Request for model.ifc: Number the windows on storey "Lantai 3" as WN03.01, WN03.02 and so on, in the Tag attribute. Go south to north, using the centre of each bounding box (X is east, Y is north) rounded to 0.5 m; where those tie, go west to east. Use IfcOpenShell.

First a look at what the model holds.

```python
import ifcopenshell
import ifcopenshell.util.element
import ifcopenshell.util.placement

model = ifcopenshell.open("model.ifc")
print(model.schema)
storey = next(s for s in model.by_type("IfcBuildingStorey") if s.Name == "Lantai 3")
windows = [e for e in ifcopenshell.util.element.get_decomposition(storey) if e.is_a("IfcWindow")]
for e in sorted(windows, key=lambda e: e.id()):
    origin = ifcopenshell.util.placement.get_local_placement(e.ObjectPlacement)[:3, 3]
    print(e.id(), e.Tag, e.Name, origin.round(2) + 0.0, sep=" | ")
```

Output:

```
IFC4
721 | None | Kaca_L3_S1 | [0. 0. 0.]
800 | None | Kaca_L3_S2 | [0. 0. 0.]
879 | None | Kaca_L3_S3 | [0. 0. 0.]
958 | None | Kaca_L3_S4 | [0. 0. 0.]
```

```python
import ifcopenshell
import ifcopenshell.geom
import ifcopenshell.util.element
import ifcopenshell.util.shape

model = ifcopenshell.open("model.ifc")
settings = ifcopenshell.geom.settings()
settings.set("use-world-coords", True)


def centre(element):
    shape = ifcopenshell.geom.create_shape(settings, element)
    return ifcopenshell.util.shape.get_bbox_centroid(shape.geometry)


storey = next(s for s in model.by_type("IfcBuildingStorey") if s.Name == "Lantai 3")
windows = [e for e in ifcopenshell.util.element.get_decomposition(storey) if e.is_a("IfcWindow")]

# Insertion points can sit at a corner or the storey origin, so sort by the geometry (in metres).
centres = {e: centre(e) for e in windows}
windows.sort(key=lambda e: (round(centres[e][1] / 0.5), centres[e][0]))

for i, e in enumerate(windows, start=1):
    number = f"WN03.{i:02d}"
    e.Tag = number
    print(e.id(), number)

model.write("model-out.ifc")
```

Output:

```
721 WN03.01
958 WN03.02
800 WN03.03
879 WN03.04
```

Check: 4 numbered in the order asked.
